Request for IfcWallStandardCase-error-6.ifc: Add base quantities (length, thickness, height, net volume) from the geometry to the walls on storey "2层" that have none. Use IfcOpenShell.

First a look at what the model holds.

```python
import ifcopenshell
import ifcopenshell.util.element
import ifcopenshell.util.unit

model = ifcopenshell.open("IfcWallStandardCase-error-6.ifc")
print(model.schema)
for unit_type in ("LENGTHUNIT", "AREAUNIT", "VOLUMEUNIT"):
    print(unit_type, ifcopenshell.util.unit.calculate_unit_scale(model, unit_type))
storey = next(s for s in model.by_type("IfcBuildingStorey") if s.Name == "2层")
walls = [e for e in ifcopenshell.util.element.get_decomposition(storey) if e.is_a("IfcWall")]
for e in sorted(walls, key=lambda e: e.id()):
    print(e.id(), e.is_a(), e.Name, list(ifcopenshell.util.element.get_psets(e, qtos_only=True)), sep=" | ")
```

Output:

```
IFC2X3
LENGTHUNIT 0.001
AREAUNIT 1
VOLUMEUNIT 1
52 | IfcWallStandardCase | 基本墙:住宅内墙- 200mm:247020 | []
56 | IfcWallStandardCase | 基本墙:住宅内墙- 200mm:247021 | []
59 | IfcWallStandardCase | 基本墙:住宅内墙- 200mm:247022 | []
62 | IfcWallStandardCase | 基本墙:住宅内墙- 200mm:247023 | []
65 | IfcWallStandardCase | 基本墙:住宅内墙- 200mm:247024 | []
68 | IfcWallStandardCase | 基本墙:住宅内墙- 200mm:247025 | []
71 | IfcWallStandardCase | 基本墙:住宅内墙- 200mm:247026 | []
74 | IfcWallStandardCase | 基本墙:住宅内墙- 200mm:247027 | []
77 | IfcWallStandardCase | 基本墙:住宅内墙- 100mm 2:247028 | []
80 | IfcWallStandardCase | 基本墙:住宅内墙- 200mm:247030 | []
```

```python
import ifcopenshell
import ifcopenshell.api.pset
import ifcopenshell.geom
import ifcopenshell.util.element
import ifcopenshell.util.shape
import ifcopenshell.util.unit

model = ifcopenshell.open("IfcWallStandardCase-error-6.ifc")
unit_scale = ifcopenshell.util.unit.calculate_unit_scale(model)
volume_scale = ifcopenshell.util.unit.calculate_unit_scale(model, "VOLUMEUNIT")
settings = ifcopenshell.geom.settings()

storey = next(s for s in model.by_type("IfcBuildingStorey") if s.Name == "2层")
walls = [e for e in ifcopenshell.util.element.get_decomposition(storey) if e.is_a("IfcWall")]

for e in sorted(walls, key=lambda e: e.id()):
    if ifcopenshell.util.element.get_psets(e, qtos_only=True, should_inherit=False):
        continue
    # Geometry comes back in metres, in the element's own axes.
    shape = ifcopenshell.geom.create_shape(settings, e)
    values = {
        "Length": ifcopenshell.util.shape.get_x(shape.geometry) / unit_scale,
        "Width": ifcopenshell.util.shape.get_y(shape.geometry) / unit_scale,
        "Height": ifcopenshell.util.shape.get_z(shape.geometry) / unit_scale,
        "NetVolume": ifcopenshell.util.shape.get_volume(shape.geometry) / volume_scale,
    }
    qto = ifcopenshell.api.pset.add_qto(model, product=e, name="BaseQuantities")
    ifcopenshell.api.pset.edit_qto(model, qto=qto, properties=values)
    print(e.id(), {k: round(v, 3) for k, v in values.items()})

model.write("IfcWallStandardCase-error-6_edited.ifc")
```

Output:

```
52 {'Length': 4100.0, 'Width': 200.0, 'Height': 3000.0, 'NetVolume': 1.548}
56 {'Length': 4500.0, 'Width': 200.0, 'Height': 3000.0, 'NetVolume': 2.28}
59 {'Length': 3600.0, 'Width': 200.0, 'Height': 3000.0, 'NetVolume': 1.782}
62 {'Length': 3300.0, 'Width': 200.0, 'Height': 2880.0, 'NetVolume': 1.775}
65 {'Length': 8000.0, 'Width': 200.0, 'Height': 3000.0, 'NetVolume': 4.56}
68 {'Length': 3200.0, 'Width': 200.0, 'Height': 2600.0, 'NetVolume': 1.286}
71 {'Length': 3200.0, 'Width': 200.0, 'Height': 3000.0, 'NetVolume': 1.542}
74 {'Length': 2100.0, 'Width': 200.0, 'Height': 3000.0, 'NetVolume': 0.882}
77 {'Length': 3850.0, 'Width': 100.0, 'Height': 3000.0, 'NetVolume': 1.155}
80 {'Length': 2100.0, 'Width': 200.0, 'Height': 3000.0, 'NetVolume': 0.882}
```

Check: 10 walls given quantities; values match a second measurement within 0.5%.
